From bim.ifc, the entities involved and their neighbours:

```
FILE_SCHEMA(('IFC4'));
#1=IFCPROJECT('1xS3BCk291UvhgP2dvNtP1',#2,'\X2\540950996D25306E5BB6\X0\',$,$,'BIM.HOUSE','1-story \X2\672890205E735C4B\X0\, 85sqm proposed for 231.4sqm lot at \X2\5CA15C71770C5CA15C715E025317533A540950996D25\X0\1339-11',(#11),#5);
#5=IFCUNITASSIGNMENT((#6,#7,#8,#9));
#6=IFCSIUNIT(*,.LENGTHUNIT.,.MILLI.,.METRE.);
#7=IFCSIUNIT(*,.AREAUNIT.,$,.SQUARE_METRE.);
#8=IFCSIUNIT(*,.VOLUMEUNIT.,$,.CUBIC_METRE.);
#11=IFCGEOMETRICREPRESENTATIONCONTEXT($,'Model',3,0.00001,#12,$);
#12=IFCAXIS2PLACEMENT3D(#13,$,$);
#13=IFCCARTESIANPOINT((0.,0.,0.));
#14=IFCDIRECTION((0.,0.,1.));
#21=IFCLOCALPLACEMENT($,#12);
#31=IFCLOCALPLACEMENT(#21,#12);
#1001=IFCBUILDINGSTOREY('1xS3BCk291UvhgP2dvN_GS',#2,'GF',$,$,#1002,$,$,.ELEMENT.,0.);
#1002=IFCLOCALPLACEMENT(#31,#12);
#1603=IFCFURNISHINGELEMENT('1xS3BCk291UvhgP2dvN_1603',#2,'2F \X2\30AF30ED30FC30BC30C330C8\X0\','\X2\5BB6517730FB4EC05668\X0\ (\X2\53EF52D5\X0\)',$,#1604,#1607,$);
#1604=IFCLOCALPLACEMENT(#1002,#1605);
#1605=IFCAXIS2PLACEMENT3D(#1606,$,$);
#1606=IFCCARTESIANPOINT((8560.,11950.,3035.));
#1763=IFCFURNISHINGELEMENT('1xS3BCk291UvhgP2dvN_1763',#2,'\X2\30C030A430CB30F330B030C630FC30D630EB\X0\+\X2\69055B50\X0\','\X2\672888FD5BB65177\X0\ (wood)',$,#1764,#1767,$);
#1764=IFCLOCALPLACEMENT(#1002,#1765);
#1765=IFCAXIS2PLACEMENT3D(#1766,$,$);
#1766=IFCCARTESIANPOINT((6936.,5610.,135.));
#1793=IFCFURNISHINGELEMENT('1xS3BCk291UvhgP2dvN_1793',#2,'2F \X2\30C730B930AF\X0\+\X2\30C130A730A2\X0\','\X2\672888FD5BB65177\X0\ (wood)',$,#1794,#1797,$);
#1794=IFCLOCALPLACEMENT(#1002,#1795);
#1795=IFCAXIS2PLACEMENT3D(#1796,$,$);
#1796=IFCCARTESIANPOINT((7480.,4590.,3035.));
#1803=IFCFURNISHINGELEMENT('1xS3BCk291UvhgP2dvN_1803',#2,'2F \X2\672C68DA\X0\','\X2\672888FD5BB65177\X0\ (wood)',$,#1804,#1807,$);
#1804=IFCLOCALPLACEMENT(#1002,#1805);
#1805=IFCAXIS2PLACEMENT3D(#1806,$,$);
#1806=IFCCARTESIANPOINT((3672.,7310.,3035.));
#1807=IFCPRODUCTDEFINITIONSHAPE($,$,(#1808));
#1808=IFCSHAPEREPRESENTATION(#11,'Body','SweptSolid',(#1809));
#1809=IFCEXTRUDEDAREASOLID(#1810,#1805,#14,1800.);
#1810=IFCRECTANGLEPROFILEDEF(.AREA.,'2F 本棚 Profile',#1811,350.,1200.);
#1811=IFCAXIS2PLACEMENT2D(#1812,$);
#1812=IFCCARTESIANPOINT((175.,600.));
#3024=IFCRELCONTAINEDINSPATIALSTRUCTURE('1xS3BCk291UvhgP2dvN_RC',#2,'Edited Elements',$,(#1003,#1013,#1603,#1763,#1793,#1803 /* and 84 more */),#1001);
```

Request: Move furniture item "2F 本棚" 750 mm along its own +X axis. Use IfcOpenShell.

```python
import ifcopenshell
import ifcopenshell.api.geometry
import ifcopenshell.util.placement

model = ifcopenshell.open("bim.ifc")

item = model.by_guid("1xS3BCk291UvhgP2dvN_1803")
matrix = ifcopenshell.util.placement.get_local_placement(item.ObjectPlacement)
matrix[:3, 3] += matrix[:3, 0] * 750.0
ifcopenshell.api.geometry.edit_object_placement(model, product=item, matrix=matrix, is_si=False)

print(ifcopenshell.util.placement.get_local_placement(item.ObjectPlacement).round(3) + 0.0)

model.write("bim_edited.ifc")
```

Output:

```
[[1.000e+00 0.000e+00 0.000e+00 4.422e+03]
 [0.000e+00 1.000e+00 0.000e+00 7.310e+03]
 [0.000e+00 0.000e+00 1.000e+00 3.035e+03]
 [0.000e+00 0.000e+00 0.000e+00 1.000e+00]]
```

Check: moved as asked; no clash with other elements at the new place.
